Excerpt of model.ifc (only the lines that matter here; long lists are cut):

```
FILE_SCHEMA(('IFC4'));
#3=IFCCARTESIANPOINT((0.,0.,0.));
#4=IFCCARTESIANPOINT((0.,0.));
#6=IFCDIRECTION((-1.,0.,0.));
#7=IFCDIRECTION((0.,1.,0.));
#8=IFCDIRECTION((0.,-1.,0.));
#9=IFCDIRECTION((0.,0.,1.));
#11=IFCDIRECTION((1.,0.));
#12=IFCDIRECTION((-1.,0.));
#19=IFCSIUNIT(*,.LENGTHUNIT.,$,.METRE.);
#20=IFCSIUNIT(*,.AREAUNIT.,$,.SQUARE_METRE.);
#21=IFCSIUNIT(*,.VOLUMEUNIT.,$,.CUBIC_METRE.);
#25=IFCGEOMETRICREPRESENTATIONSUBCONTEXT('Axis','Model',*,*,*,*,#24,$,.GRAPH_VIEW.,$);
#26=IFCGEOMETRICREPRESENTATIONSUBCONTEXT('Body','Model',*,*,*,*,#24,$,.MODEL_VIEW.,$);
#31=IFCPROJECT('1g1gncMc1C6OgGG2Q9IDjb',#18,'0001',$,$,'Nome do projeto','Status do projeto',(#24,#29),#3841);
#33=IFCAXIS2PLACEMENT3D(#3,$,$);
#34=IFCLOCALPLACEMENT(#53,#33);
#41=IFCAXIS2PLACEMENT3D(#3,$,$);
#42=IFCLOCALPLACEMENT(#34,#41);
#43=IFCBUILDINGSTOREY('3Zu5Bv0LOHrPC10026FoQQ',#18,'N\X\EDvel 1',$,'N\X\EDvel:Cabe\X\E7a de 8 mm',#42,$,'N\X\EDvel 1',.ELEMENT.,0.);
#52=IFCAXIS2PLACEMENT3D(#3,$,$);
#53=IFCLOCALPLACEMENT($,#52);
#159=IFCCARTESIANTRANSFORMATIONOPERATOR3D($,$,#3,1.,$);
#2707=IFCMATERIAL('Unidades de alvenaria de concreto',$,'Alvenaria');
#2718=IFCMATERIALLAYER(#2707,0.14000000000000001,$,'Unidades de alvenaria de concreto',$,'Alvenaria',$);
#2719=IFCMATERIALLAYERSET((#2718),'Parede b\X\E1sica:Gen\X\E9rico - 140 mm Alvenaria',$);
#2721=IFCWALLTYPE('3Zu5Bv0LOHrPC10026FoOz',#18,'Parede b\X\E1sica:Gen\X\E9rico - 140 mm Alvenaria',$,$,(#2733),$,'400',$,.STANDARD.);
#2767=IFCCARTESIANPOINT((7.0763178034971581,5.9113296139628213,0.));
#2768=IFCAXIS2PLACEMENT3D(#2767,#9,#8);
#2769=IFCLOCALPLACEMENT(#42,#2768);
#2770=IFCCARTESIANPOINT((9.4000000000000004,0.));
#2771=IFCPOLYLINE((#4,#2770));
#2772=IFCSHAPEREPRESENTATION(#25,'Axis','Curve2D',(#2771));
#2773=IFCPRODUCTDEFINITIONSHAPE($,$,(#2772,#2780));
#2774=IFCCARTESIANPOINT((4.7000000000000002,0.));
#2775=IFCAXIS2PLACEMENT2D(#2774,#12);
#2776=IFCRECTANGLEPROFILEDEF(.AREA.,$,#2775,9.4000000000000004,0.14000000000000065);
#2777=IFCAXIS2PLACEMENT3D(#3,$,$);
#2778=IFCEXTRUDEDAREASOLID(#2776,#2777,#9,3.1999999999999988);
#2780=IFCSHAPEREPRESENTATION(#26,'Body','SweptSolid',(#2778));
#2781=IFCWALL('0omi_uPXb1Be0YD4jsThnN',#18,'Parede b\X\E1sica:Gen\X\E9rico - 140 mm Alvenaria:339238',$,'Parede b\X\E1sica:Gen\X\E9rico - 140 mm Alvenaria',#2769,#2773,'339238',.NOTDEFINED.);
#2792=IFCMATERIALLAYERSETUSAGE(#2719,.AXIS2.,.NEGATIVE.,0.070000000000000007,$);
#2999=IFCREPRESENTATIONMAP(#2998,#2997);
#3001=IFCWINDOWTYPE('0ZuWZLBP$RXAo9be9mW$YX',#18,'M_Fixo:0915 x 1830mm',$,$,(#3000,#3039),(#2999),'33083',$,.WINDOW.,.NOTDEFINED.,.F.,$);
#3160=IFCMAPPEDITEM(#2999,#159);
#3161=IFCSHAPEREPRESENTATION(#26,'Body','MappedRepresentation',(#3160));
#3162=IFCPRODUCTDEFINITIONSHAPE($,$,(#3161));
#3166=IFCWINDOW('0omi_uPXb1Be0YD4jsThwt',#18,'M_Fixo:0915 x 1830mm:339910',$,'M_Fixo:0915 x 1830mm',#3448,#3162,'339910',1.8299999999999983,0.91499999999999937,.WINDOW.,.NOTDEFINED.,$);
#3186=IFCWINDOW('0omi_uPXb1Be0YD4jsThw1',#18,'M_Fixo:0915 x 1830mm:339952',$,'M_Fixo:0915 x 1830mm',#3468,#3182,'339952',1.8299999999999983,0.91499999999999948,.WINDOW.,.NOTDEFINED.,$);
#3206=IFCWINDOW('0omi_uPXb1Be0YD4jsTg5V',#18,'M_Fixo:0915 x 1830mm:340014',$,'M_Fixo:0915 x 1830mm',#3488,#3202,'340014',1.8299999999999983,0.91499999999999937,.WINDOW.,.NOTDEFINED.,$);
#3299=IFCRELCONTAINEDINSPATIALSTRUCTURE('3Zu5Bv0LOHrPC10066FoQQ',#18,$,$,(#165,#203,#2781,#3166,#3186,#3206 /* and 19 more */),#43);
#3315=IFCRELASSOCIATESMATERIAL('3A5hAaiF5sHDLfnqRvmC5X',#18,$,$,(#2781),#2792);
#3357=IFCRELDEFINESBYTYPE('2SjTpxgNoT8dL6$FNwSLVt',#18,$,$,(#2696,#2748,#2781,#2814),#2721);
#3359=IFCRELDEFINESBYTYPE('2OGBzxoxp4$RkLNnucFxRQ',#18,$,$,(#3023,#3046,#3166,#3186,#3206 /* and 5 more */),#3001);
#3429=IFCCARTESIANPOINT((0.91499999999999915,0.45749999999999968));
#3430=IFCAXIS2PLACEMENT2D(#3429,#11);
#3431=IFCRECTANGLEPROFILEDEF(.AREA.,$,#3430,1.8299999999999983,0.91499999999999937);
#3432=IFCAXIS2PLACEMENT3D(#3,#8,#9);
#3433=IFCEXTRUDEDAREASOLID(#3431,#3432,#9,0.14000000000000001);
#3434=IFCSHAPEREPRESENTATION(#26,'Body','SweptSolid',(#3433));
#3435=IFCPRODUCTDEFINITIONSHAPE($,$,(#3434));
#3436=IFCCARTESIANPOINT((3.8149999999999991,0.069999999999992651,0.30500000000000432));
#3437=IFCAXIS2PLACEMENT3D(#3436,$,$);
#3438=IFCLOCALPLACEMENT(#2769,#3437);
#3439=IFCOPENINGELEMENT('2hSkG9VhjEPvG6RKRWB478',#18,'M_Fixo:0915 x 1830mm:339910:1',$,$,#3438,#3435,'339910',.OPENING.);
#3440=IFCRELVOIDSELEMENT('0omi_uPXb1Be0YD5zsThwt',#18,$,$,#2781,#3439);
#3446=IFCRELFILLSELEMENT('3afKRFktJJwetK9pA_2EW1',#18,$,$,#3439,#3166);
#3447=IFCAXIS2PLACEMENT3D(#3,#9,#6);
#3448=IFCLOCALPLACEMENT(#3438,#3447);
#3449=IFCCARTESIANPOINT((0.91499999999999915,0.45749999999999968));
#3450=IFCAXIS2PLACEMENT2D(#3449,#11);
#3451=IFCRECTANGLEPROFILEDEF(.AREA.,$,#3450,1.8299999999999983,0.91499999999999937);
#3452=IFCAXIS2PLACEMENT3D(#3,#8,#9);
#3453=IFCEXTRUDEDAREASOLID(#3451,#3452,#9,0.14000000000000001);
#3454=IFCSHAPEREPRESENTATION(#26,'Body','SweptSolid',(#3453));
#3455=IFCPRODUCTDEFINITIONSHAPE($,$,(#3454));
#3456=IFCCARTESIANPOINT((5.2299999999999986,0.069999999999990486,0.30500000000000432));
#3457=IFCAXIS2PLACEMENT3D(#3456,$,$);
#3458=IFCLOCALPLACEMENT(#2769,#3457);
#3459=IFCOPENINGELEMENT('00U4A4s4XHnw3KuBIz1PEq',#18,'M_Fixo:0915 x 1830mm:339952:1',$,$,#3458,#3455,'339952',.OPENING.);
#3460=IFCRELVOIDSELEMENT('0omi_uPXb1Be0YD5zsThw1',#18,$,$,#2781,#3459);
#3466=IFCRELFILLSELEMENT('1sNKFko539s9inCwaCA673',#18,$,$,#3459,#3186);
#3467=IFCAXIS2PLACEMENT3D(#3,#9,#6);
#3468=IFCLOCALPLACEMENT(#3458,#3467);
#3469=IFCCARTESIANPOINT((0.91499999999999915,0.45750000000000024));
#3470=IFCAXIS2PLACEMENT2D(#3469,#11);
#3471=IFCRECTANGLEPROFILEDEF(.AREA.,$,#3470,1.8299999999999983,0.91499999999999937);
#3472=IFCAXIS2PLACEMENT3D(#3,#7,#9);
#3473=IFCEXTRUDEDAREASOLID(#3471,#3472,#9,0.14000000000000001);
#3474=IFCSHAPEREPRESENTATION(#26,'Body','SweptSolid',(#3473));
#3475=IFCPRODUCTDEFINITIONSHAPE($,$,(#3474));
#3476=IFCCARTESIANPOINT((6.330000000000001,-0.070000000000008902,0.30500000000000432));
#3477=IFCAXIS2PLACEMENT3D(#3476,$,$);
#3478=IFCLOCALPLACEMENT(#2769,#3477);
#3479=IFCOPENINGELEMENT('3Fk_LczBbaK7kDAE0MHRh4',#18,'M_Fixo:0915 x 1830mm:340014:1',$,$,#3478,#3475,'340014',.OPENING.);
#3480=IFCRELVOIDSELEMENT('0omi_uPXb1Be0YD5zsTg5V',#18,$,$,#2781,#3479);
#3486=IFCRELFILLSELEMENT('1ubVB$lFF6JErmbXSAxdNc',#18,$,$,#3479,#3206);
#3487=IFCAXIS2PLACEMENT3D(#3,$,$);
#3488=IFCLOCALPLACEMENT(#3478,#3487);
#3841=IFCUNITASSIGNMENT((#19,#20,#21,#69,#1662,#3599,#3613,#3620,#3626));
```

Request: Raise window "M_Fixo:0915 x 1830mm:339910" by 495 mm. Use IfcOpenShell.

```python
import numpy as np
import ifcopenshell
import ifcopenshell.api.geometry
import ifcopenshell.util.placement
import ifcopenshell.util.unit

model = ifcopenshell.open("model.ifc")
unit_scale = ifcopenshell.util.unit.calculate_unit_scale(model)

window = model.by_id(3166)
opening = window.FillsVoids[0].RelatingOpeningElement
dz = 0.495 / unit_scale

shift = np.array([0.0, 0.0, dz])
# The window is placed relative to its opening, so it follows when the opening moves.
matrix = ifcopenshell.util.placement.get_local_placement(opening.ObjectPlacement)
matrix[:3, 3] += shift
ifcopenshell.api.geometry.edit_object_placement(
    model, product=opening, matrix=matrix, is_si=False, should_transform_children=True
)

print(f"moved by {dz * unit_scale:+.3f} m")

model.write("model-out.ifc")
```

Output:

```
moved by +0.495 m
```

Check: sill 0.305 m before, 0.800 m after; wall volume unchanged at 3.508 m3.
